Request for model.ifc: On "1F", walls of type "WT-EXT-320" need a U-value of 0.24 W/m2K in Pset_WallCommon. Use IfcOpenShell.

First a look at what the model holds.

```python
import ifcopenshell
import ifcopenshell.util.element

model = ifcopenshell.open("model.ifc")
print(model.schema)
storey = next(s for s in model.by_type("IfcBuildingStorey") if s.Name == "1F")
walls = [e for e in ifcopenshell.util.element.get_decomposition(storey) if e.is_a("IfcWall")]
seen = {}
for e in walls:
    element_type = ifcopenshell.util.element.get_type(e)
    key = (element_type.Name if element_type != e and element_type else None, ifcopenshell.util.element.get_pset(e, "Pset_WallCommon", "ThermalTransmittance"))
    seen[key] = seen.get(key, 0) + 1
for (name, value), count in sorted(seen.items(), key=str):
    print(count, "x", name, "|", value)
```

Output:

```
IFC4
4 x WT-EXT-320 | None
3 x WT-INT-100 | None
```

```python
import ifcopenshell
import ifcopenshell.api.pset
import ifcopenshell.util.element

model = ifcopenshell.open("model.ifc")

storey = next(s for s in model.by_type("IfcBuildingStorey") if s.Name == "1F")
walls = [e for e in ifcopenshell.util.element.get_decomposition(storey) if e.is_a("IfcWall")]

count = 0
for e in walls:
    element_type = ifcopenshell.util.element.get_type(e)
    if element_type in (None, e) or element_type.Name != "WT-EXT-320":
        continue
    # add_pset returns the element's existing set when there is one.
    pset = ifcopenshell.api.pset.add_pset(model, product=e, name="Pset_WallCommon")
    ifcopenshell.api.pset.edit_pset(model, pset=pset, properties={"ThermalTransmittance": 0.24})
    count += 1

print(count, "walls updated")

model.write("model-out.ifc")
```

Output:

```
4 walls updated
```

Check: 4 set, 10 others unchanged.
